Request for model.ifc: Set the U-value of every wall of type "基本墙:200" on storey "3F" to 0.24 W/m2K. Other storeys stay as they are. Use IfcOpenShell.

First a look at what the model holds.

```python
import ifcopenshell
import ifcopenshell.util.element

model = ifcopenshell.open("model.ifc")
print(model.schema)
storey = next(s for s in model.by_type("IfcBuildingStorey") if s.Name == "3F")
walls = [e for e in ifcopenshell.util.element.get_decomposition(storey) if e.is_a("IfcWall")]
seen = {}
for e in walls:
    element_type = ifcopenshell.util.element.get_type(e)
    key = (element_type.Name if element_type != e and element_type else None, ifcopenshell.util.element.get_pset(e, "Pset_WallCommon", "ThermalTransmittance"))
    seen[key] = seen.get(key, 0) + 1
for (name, value), count in sorted(seen.items(), key=str):
    print(count, "x", name, "|", value)
```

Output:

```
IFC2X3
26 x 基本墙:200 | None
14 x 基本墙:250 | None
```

```python
import ifcopenshell
import ifcopenshell.api.pset
import ifcopenshell.util.element

model = ifcopenshell.open("model.ifc")

storey = next(s for s in model.by_type("IfcBuildingStorey") if s.Name == "3F")
walls = [e for e in ifcopenshell.util.element.get_decomposition(storey) if e.is_a("IfcWall")]

count = 0
for e in walls:
    element_type = ifcopenshell.util.element.get_type(e)
    if element_type in (None, e) or element_type.Name != "基本墙:200":
        continue
    # add_pset returns the element's existing set when there is one.
    pset = ifcopenshell.api.pset.add_pset(model, product=e, name="Pset_WallCommon")
    ifcopenshell.api.pset.edit_pset(model, pset=pset, properties={"ThermalTransmittance": 0.24})
    count += 1

print(count, "walls updated")

model.write("model_edited.ifc")
```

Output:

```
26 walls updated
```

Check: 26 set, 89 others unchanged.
